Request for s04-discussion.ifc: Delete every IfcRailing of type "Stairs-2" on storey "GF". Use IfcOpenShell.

First a look at what the model holds.

```python
import ifcopenshell
import ifcopenshell.util.element

model = ifcopenshell.open("s04-discussion.ifc")
print(model.schema)
storey = next(s for s in model.by_type("IfcBuildingStorey") if s.Name == "GF")
railings = [e for e in ifcopenshell.util.element.get_decomposition(storey) if e.is_a("IfcRailing")]
seen = {}
for e in railings:
    element_type = ifcopenshell.util.element.get_type(e)
    name = element_type.Name if element_type not in (None, e) else None
    seen[name] = seen.get(name, 0) + 1
for name, count in sorted(seen.items(), key=str):
    print(count, "x", name)
```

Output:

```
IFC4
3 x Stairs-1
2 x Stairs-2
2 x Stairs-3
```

```python
import ifcopenshell
import ifcopenshell.api.root
import ifcopenshell.util.element

model = ifcopenshell.open("s04-discussion.ifc")

storey = next(s for s in model.by_type("IfcBuildingStorey") if s.Name == "GF")
railings = [e for e in ifcopenshell.util.element.get_decomposition(storey) if e.is_a("IfcRailing")]
targets = [e for e in railings if (t := ifcopenshell.util.element.get_type(e)) not in (None, e) and t.Name == "Stairs-2"]

for e in targets:
    ifcopenshell.api.root.remove_product(model, product=e)
print(len(targets), "removed")

model.write("s04-discussion-out.ifc")
```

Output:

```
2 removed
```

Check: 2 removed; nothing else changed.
